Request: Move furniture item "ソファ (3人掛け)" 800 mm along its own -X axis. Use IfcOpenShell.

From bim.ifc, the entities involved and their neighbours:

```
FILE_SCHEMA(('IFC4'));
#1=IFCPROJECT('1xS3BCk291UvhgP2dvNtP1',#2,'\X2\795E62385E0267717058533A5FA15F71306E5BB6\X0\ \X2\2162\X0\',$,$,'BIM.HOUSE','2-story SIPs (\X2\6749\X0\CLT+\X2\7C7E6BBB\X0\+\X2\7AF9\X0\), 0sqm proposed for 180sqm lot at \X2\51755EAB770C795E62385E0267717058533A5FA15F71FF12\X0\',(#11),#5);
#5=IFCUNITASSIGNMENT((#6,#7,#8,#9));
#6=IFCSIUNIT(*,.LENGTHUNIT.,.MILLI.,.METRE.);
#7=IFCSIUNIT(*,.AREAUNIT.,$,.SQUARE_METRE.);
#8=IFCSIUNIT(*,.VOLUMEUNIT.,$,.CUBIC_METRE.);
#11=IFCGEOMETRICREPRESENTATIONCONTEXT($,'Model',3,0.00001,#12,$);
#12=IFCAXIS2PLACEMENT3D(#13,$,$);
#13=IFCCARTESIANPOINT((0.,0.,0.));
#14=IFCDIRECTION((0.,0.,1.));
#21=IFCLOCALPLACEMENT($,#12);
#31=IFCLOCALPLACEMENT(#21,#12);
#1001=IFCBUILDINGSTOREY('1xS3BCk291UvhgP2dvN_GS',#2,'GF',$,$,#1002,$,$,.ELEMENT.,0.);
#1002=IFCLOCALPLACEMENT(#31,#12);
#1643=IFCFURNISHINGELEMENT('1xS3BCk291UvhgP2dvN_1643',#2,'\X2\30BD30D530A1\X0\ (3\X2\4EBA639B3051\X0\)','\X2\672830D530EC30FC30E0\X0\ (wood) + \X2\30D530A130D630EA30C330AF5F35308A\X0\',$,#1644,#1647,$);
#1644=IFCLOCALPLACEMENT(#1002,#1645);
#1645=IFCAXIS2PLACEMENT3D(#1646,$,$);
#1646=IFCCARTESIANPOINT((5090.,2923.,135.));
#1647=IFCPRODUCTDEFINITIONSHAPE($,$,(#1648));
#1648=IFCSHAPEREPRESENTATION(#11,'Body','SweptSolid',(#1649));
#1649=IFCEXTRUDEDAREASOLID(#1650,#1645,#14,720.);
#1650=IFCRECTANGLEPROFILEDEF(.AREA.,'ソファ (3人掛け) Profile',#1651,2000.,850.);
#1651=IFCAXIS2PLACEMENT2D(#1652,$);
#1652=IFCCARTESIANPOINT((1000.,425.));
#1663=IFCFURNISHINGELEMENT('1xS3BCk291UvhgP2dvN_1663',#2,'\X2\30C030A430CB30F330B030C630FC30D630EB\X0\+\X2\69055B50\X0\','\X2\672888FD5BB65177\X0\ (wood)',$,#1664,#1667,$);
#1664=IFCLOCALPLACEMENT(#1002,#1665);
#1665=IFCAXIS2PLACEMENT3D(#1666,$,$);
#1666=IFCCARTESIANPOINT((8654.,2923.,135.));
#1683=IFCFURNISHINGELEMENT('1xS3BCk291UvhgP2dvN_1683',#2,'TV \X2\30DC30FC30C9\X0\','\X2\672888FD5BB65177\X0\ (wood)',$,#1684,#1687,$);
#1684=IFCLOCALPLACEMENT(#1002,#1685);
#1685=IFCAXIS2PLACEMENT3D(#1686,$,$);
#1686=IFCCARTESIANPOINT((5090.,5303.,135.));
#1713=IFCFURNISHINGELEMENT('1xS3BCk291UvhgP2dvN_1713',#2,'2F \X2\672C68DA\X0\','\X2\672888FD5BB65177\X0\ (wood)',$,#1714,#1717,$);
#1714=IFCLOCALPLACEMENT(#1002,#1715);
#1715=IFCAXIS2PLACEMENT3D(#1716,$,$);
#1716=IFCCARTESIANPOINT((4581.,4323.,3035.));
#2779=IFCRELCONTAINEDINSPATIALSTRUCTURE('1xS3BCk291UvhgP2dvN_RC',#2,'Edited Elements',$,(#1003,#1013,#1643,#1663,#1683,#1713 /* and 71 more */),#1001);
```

```python
import ifcopenshell
import ifcopenshell.api.geometry
import ifcopenshell.util.placement
import ifcopenshell.util.unit

model = ifcopenshell.open("bim.ifc")
unit_scale = ifcopenshell.util.unit.calculate_unit_scale(model)

item = model.by_guid("1xS3BCk291UvhgP2dvN_1643")
matrix = ifcopenshell.util.placement.get_local_placement(item.ObjectPlacement)
matrix[:3, 3] -= matrix[:3, 0] * 0.8 / unit_scale
ifcopenshell.api.geometry.edit_object_placement(model, product=item, matrix=matrix, is_si=False)

print(ifcopenshell.util.placement.get_local_placement(item.ObjectPlacement).round(3) + 0.0)

model.write("bim_v2.ifc")
```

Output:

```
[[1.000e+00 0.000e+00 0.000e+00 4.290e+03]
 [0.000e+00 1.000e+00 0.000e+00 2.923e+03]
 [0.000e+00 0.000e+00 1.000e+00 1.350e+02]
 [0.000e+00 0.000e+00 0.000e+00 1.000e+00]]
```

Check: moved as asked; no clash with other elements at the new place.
